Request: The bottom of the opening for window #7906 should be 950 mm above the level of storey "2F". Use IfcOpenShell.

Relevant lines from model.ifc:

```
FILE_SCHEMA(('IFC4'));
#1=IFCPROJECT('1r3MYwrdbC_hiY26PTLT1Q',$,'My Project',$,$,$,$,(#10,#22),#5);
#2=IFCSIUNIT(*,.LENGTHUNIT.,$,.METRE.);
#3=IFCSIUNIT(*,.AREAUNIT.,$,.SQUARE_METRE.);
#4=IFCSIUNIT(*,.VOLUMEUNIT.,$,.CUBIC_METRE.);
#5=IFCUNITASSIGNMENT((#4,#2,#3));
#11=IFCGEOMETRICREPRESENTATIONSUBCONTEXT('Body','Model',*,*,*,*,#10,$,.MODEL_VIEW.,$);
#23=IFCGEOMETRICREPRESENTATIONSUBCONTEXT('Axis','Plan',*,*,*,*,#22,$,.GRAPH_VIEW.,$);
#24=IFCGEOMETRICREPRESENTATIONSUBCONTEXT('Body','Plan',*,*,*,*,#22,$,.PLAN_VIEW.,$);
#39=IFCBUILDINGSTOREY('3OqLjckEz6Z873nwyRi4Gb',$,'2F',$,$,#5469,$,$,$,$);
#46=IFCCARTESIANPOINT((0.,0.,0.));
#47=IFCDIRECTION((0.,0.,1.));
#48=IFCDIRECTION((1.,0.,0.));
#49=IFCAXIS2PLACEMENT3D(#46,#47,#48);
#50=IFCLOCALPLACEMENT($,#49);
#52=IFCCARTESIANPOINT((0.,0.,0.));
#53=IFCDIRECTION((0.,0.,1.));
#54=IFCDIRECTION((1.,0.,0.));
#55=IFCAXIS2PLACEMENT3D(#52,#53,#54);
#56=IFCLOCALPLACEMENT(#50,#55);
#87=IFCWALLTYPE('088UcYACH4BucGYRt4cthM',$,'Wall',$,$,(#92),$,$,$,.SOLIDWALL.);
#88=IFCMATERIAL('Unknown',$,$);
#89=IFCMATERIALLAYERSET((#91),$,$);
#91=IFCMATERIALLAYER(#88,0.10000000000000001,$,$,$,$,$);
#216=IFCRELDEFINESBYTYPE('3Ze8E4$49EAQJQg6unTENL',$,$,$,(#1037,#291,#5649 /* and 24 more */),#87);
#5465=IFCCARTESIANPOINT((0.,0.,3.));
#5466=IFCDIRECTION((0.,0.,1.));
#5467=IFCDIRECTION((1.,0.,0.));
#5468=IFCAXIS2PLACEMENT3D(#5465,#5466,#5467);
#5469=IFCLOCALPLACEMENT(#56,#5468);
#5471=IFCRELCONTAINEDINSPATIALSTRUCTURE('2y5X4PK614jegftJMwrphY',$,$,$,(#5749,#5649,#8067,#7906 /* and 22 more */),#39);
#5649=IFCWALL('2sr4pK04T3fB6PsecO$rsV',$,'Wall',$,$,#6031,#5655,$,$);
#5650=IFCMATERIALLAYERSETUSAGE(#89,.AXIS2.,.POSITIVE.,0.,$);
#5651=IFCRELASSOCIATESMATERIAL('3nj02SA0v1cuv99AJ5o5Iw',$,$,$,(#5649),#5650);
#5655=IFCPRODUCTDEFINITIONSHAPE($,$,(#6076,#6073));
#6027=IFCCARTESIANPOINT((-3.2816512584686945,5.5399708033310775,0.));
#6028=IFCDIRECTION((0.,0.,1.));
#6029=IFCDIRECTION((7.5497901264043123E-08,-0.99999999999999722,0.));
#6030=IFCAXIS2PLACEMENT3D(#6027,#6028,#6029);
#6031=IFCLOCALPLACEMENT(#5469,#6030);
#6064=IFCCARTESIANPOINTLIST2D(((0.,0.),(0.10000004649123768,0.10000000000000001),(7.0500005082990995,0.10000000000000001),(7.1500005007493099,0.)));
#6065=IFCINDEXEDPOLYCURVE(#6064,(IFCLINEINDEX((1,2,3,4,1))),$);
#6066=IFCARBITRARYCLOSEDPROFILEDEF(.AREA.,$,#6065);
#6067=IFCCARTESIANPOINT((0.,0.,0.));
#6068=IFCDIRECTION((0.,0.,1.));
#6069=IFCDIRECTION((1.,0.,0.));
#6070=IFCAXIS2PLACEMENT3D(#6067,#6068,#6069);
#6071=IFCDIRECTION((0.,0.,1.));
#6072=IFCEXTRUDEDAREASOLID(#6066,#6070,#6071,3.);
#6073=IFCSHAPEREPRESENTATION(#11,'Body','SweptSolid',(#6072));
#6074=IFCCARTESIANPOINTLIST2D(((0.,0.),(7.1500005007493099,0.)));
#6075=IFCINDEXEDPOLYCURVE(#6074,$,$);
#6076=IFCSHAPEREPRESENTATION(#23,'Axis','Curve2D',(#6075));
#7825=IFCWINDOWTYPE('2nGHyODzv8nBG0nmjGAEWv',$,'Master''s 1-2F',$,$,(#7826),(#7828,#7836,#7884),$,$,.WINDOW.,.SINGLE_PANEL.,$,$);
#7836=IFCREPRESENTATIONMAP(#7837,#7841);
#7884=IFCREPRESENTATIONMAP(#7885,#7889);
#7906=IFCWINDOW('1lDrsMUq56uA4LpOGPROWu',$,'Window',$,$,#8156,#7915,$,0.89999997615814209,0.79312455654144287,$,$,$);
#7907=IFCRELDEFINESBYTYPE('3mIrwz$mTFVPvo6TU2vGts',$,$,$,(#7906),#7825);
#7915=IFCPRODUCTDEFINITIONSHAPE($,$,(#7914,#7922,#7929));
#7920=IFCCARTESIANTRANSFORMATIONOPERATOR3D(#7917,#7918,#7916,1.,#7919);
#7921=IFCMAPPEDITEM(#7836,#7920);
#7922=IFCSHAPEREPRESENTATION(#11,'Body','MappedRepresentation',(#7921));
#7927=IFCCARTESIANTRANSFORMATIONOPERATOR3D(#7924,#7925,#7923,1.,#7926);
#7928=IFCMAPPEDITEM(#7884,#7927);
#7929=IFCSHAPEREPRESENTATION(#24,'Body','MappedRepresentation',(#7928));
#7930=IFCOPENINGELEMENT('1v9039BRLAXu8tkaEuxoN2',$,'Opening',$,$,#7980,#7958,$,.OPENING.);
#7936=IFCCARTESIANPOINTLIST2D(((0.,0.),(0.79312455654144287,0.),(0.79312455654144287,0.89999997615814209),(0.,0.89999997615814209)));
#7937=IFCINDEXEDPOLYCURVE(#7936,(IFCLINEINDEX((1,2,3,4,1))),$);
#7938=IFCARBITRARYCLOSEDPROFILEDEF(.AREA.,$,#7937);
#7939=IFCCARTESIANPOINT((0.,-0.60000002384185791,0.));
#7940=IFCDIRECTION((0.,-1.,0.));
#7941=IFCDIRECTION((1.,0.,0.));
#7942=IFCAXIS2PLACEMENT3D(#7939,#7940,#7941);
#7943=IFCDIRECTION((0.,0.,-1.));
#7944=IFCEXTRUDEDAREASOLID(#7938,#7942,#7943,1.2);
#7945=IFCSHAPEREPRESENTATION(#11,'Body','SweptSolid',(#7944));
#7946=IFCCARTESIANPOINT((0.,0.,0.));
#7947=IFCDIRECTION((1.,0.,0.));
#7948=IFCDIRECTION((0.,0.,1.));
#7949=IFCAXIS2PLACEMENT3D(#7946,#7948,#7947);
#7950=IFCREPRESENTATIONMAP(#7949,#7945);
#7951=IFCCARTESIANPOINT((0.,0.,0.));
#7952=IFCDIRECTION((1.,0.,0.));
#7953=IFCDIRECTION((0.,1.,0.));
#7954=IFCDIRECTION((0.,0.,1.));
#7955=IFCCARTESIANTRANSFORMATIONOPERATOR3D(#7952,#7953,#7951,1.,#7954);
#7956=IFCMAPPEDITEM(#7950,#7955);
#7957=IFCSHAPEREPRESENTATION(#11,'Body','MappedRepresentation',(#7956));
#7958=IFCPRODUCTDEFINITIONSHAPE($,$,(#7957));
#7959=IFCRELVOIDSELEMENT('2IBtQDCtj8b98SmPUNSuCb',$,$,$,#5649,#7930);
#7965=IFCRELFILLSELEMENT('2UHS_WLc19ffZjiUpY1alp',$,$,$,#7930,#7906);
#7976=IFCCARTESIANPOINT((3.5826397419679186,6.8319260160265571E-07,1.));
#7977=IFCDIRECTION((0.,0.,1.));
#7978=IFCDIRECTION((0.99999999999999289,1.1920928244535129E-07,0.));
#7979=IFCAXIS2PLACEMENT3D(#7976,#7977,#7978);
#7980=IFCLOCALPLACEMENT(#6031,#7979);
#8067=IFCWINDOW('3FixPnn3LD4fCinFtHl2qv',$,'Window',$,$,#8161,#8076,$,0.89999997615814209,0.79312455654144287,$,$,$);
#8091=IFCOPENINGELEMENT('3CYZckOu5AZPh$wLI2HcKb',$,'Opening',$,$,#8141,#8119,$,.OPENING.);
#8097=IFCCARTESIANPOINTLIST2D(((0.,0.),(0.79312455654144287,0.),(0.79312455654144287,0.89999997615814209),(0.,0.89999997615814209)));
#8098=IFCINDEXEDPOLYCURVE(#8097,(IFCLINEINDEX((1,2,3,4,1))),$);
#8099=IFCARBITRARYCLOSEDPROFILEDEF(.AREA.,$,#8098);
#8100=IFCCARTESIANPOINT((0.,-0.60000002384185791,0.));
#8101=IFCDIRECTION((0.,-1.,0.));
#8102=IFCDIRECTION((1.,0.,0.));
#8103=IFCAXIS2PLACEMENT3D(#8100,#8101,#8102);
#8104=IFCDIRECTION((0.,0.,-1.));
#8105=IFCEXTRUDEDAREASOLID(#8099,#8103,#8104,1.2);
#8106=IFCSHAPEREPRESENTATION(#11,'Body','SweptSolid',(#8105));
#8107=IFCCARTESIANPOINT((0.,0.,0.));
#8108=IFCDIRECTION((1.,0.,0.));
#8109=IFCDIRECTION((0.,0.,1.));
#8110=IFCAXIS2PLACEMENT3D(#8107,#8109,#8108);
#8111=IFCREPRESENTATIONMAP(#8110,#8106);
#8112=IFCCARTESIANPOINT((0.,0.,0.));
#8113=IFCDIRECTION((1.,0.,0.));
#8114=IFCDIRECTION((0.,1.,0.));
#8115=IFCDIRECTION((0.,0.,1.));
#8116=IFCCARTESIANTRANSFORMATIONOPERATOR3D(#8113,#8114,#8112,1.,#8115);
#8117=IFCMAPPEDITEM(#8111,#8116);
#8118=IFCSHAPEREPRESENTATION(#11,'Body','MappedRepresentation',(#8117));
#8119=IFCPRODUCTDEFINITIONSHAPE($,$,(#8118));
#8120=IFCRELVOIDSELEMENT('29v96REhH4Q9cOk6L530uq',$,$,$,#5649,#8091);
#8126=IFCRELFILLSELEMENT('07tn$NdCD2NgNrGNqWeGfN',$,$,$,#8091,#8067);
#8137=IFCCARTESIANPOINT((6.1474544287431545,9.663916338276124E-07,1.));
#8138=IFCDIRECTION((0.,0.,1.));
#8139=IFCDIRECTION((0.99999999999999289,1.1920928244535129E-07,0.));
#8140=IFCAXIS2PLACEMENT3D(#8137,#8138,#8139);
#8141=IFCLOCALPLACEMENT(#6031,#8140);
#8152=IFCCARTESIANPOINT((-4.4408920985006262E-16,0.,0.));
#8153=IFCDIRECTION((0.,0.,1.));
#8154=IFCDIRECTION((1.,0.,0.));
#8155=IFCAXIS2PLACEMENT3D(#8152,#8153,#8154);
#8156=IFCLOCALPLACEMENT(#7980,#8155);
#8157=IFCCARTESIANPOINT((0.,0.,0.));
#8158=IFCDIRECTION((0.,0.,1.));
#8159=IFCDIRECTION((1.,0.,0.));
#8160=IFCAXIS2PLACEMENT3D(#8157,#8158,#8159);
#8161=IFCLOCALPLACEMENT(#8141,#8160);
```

```python
import numpy as np
import ifcopenshell
import ifcopenshell.api.geometry
import ifcopenshell.geom
import ifcopenshell.util.element
import ifcopenshell.util.placement
import ifcopenshell.util.shape
import ifcopenshell.util.unit

model = ifcopenshell.open("model.ifc")
unit_scale = ifcopenshell.util.unit.calculate_unit_scale(model)

window = model.by_guid("1lDrsMUq56uA4LpOGPROWu")
opening = window.FillsVoids[0].RelatingOpeningElement
storey = ifcopenshell.util.element.get_container(window, ifc_class="IfcBuildingStorey")
level = ifcopenshell.util.placement.get_local_placement(storey.ObjectPlacement)[2, 3]

# The opening's origin need not be at the sill, so measure its lowest point.
shape = ifcopenshell.geom.create_shape(ifcopenshell.geom.settings(), opening)
bottom = ifcopenshell.util.shape.get_shape_bottom_elevation(shape, shape.geometry) / unit_scale
dz = level + 0.95 - bottom

shift = np.array([0.0, 0.0, dz])
# The window is placed relative to its opening, so it follows when the opening moves.
matrix = ifcopenshell.util.placement.get_local_placement(opening.ObjectPlacement)
matrix[:3, 3] += shift
ifcopenshell.api.geometry.edit_object_placement(
    model, product=opening, matrix=matrix, is_si=False, should_transform_children=True
)

print(f"moved by {dz * unit_scale:+.3f} m")

model.write("model_edited.ifc")
```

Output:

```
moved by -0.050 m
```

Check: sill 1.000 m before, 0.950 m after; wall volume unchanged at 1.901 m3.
